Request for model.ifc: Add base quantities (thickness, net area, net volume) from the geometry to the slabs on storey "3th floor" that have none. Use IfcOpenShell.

First a look at what the model holds.

```python
import ifcopenshell
import ifcopenshell.util.element
import ifcopenshell.util.unit

model = ifcopenshell.open("model.ifc")
print(model.schema)
for unit_type in ("LENGTHUNIT", "AREAUNIT", "VOLUMEUNIT"):
    print(unit_type, ifcopenshell.util.unit.calculate_unit_scale(model, unit_type))
storey = next(s for s in model.by_type("IfcBuildingStorey") if s.Name == "3th floor")
slabs = [e for e in ifcopenshell.util.element.get_decomposition(storey) if e.is_a("IfcSlab")]
for e in sorted(slabs, key=lambda e: e.id()):
    print(e.id(), e.is_a(), e.Name, list(ifcopenshell.util.element.get_psets(e, qtos_only=True)), sep=" | ")
```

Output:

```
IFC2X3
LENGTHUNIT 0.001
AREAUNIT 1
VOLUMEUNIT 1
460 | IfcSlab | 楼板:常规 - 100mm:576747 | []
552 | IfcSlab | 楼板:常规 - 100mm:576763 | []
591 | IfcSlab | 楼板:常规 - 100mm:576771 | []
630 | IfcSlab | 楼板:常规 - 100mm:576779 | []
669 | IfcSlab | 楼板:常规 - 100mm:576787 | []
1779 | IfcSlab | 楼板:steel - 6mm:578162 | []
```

```python
import ifcopenshell
import ifcopenshell.api.pset
import ifcopenshell.geom
import ifcopenshell.util.element
import ifcopenshell.util.shape
import ifcopenshell.util.unit

model = ifcopenshell.open("model.ifc")
unit_scale = ifcopenshell.util.unit.calculate_unit_scale(model)
area_scale = ifcopenshell.util.unit.calculate_unit_scale(model, "AREAUNIT")
volume_scale = ifcopenshell.util.unit.calculate_unit_scale(model, "VOLUMEUNIT")
settings = ifcopenshell.geom.settings()

storey = next(s for s in model.by_type("IfcBuildingStorey") if s.Name == "3th floor")
slabs = [e for e in ifcopenshell.util.element.get_decomposition(storey) if e.is_a("IfcSlab")]

for e in sorted(slabs, key=lambda e: e.id()):
    if ifcopenshell.util.element.get_psets(e, qtos_only=True, should_inherit=False):
        continue
    # Geometry comes back in metres, in the element's own axes.
    shape = ifcopenshell.geom.create_shape(settings, e)
    values = {
        "Width": ifcopenshell.util.shape.get_z(shape.geometry) / unit_scale,
        "NetArea": ifcopenshell.util.shape.get_footprint_area(shape.geometry) / area_scale,
        "NetVolume": ifcopenshell.util.shape.get_volume(shape.geometry) / volume_scale,
    }
    qto = ifcopenshell.api.pset.add_qto(model, product=e, name="BaseQuantities")
    ifcopenshell.api.pset.edit_qto(model, qto=qto, properties=values)
    print(e.id(), {k: round(v, 3) for k, v in values.items()})

model.write("model_updated.ifc")
```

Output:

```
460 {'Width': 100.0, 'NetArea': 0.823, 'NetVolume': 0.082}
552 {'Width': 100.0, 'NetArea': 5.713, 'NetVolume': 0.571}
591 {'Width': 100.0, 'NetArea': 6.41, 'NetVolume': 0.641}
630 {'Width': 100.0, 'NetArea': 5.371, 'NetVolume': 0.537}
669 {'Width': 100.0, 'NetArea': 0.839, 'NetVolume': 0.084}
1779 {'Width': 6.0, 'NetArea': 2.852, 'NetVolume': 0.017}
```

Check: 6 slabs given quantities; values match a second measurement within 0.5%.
